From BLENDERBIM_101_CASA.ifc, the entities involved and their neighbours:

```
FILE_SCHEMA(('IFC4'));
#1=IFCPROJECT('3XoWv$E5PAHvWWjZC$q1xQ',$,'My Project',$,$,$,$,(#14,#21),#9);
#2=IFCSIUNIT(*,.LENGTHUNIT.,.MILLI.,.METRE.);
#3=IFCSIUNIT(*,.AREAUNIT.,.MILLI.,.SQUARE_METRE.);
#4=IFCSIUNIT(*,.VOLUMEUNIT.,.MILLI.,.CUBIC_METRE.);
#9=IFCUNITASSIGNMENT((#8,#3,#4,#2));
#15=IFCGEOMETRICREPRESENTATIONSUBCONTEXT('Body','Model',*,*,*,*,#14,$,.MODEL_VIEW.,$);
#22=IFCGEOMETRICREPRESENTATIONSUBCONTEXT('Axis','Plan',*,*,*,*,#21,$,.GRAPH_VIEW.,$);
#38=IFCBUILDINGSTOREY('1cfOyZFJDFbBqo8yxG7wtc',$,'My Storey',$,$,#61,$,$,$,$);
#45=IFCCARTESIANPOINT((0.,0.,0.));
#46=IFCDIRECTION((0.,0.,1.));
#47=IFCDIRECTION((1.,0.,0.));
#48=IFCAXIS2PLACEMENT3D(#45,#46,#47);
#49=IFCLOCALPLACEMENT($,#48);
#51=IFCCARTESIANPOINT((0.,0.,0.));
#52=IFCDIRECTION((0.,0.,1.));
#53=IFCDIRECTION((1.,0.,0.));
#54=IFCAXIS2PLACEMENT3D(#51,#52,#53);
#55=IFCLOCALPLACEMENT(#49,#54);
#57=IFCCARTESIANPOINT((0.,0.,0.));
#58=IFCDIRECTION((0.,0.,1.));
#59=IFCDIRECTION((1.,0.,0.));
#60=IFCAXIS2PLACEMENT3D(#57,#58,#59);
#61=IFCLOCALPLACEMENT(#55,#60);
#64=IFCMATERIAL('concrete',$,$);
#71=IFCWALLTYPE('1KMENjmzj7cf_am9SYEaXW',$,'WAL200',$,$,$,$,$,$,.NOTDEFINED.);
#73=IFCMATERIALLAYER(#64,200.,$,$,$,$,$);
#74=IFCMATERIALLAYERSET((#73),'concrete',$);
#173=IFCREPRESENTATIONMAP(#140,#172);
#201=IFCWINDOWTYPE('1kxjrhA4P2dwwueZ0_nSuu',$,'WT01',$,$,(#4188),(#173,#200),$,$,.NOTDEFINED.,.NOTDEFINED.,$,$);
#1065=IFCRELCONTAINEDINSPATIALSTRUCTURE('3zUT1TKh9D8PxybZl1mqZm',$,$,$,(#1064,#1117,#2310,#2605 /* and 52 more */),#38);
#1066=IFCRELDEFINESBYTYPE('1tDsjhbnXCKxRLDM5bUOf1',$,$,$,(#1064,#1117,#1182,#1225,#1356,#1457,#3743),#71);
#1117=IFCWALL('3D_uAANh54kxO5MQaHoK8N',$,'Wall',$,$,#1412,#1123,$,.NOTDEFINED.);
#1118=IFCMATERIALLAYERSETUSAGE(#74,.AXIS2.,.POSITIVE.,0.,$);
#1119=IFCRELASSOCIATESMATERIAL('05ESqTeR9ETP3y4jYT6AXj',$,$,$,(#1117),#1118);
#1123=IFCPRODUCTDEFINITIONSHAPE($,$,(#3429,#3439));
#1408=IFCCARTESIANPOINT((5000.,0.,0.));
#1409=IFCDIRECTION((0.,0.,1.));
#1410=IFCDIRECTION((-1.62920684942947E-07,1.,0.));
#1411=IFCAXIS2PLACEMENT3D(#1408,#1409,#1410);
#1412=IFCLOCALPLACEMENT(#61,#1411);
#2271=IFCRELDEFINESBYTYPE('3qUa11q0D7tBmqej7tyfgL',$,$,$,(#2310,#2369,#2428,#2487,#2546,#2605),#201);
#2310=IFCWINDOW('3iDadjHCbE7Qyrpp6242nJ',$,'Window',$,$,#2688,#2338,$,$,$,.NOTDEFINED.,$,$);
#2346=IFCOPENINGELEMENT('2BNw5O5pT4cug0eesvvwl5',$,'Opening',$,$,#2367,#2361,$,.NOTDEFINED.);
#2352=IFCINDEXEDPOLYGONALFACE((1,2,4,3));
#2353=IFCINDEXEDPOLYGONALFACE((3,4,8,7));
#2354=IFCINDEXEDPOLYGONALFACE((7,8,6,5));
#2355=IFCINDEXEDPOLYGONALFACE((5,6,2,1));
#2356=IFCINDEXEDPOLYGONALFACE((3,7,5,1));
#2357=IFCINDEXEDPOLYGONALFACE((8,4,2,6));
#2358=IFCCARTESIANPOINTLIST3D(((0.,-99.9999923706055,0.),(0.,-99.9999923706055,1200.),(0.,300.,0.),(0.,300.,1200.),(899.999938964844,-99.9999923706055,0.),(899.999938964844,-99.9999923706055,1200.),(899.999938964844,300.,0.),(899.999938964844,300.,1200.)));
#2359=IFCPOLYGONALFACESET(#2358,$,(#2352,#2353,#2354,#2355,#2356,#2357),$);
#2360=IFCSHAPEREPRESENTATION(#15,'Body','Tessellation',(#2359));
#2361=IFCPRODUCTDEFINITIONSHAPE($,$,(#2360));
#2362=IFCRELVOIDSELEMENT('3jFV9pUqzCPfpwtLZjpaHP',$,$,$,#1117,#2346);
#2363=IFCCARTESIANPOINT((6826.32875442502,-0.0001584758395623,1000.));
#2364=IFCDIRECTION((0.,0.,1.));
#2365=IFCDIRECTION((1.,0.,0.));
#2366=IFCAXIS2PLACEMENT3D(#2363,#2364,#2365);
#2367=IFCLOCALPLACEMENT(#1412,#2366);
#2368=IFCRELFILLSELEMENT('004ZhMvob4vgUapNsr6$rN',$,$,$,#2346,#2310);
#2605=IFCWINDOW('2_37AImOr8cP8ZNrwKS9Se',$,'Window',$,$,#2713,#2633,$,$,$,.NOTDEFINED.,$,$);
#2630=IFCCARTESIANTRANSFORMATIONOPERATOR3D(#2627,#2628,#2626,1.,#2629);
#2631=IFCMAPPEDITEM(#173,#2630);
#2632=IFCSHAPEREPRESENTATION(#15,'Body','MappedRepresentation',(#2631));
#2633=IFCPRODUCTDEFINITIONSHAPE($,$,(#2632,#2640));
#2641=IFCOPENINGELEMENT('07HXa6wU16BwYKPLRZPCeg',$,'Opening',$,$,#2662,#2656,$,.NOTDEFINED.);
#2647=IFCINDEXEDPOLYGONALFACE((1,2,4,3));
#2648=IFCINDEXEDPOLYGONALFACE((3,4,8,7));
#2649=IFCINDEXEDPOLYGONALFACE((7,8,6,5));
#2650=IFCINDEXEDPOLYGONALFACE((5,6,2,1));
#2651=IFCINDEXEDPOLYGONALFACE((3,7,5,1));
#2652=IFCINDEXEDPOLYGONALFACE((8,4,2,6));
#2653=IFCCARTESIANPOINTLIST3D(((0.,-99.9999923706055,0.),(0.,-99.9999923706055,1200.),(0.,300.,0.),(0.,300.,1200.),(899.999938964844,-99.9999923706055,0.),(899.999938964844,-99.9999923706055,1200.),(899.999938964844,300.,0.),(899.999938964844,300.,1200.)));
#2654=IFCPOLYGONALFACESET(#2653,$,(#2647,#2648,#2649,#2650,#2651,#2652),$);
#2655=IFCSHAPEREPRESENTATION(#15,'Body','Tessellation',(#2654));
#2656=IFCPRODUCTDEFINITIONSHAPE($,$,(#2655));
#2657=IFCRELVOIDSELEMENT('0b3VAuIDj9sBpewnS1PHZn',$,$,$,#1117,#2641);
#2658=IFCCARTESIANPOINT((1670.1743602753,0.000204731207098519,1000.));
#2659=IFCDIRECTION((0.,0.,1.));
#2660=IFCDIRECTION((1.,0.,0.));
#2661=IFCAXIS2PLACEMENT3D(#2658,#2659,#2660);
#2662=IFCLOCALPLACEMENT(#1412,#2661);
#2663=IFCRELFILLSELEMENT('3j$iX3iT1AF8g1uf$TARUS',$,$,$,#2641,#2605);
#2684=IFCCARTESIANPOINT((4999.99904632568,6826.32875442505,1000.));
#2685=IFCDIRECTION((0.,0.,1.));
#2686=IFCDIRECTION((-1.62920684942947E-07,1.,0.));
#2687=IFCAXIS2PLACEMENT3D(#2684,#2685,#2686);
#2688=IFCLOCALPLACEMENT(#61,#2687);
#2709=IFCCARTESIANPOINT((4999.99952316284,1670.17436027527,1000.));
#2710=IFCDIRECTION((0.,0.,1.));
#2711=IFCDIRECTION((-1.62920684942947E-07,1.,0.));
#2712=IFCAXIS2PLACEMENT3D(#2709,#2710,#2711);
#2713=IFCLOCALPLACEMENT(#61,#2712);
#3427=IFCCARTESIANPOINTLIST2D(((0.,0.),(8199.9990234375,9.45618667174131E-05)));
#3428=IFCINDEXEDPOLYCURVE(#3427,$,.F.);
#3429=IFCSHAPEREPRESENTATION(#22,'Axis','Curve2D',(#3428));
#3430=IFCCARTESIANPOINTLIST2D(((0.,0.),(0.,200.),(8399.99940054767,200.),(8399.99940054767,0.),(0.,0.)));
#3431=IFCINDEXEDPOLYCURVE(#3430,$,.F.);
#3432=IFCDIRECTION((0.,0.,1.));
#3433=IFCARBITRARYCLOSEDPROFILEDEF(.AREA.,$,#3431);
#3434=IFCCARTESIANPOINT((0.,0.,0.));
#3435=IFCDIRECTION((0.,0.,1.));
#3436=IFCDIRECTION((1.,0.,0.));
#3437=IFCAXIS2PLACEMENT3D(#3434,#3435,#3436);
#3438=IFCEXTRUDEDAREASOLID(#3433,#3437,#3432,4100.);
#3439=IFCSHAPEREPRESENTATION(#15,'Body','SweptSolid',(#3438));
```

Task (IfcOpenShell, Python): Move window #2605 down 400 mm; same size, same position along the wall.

```python
import numpy as np
import ifcopenshell
import ifcopenshell.api.geometry
import ifcopenshell.util.placement
import ifcopenshell.util.unit

model = ifcopenshell.open("BLENDERBIM_101_CASA.ifc")
unit_scale = ifcopenshell.util.unit.calculate_unit_scale(model)

window = model.by_id(2605)
opening = window.FillsVoids[0].RelatingOpeningElement
dz = -0.4 / unit_scale

shift = np.array([0.0, 0.0, dz])
# The window is not placed relative to its opening, so move both.
for product in (opening, window):
    matrix = ifcopenshell.util.placement.get_local_placement(product.ObjectPlacement)
    matrix[:3, 3] += shift
    ifcopenshell.api.geometry.edit_object_placement(model, product=product, matrix=matrix, is_si=False)

print(f"moved by {dz * unit_scale:+.3f} m")

model.write("BLENDERBIM_101_CASA-out.ifc")
```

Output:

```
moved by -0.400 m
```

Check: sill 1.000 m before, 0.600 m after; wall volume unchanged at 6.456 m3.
